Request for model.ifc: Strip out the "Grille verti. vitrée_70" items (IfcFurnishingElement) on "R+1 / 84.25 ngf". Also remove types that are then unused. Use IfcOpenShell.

First a look at what the model holds.

```python
import ifcopenshell
import ifcopenshell.util.element

model = ifcopenshell.open("model.ifc")
print(model.schema)
storey = next(s for s in model.by_type("IfcBuildingStorey") if s.Name == "R+1 / 84.25 ngf")
furniture = [e for e in ifcopenshell.util.element.get_decomposition(storey) if e.is_a("IfcFurnishingElement")]
seen = {}
for e in furniture:
    element_type = ifcopenshell.util.element.get_type(e)
    name = element_type.Name if element_type not in (None, e) else None
    seen[name] = seen.get(name, 0) + 1
for name, count in sorted(seen.items(), key=str):
    print(count, "x", name)
```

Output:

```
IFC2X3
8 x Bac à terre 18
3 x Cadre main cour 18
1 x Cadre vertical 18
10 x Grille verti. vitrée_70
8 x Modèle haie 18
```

```python
import ifcopenshell
import ifcopenshell.api.root
import ifcopenshell.util.element

model = ifcopenshell.open("model.ifc")

storey = next(s for s in model.by_type("IfcBuildingStorey") if s.Name == "R+1 / 84.25 ngf")
furniture = [e for e in ifcopenshell.util.element.get_decomposition(storey) if e.is_a("IfcFurnishingElement")]
targets = [e for e in furniture if (t := ifcopenshell.util.element.get_type(e)) not in (None, e) and t.Name == "Grille verti. vitrée_70"]
types = {ifcopenshell.util.element.get_type(e) for e in targets} - {None, *targets}

for e in targets:
    ifcopenshell.api.root.remove_product(model, product=e)
print(len(targets), "removed")

unused = [t for t in types if not ifcopenshell.util.element.get_types(t)]
for t in unused:
    ifcopenshell.api.root.remove_product(model, product=t)
print(len(unused), "unused types removed")

model.write("model_updated.ifc")
```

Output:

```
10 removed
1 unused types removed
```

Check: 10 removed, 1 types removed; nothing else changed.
